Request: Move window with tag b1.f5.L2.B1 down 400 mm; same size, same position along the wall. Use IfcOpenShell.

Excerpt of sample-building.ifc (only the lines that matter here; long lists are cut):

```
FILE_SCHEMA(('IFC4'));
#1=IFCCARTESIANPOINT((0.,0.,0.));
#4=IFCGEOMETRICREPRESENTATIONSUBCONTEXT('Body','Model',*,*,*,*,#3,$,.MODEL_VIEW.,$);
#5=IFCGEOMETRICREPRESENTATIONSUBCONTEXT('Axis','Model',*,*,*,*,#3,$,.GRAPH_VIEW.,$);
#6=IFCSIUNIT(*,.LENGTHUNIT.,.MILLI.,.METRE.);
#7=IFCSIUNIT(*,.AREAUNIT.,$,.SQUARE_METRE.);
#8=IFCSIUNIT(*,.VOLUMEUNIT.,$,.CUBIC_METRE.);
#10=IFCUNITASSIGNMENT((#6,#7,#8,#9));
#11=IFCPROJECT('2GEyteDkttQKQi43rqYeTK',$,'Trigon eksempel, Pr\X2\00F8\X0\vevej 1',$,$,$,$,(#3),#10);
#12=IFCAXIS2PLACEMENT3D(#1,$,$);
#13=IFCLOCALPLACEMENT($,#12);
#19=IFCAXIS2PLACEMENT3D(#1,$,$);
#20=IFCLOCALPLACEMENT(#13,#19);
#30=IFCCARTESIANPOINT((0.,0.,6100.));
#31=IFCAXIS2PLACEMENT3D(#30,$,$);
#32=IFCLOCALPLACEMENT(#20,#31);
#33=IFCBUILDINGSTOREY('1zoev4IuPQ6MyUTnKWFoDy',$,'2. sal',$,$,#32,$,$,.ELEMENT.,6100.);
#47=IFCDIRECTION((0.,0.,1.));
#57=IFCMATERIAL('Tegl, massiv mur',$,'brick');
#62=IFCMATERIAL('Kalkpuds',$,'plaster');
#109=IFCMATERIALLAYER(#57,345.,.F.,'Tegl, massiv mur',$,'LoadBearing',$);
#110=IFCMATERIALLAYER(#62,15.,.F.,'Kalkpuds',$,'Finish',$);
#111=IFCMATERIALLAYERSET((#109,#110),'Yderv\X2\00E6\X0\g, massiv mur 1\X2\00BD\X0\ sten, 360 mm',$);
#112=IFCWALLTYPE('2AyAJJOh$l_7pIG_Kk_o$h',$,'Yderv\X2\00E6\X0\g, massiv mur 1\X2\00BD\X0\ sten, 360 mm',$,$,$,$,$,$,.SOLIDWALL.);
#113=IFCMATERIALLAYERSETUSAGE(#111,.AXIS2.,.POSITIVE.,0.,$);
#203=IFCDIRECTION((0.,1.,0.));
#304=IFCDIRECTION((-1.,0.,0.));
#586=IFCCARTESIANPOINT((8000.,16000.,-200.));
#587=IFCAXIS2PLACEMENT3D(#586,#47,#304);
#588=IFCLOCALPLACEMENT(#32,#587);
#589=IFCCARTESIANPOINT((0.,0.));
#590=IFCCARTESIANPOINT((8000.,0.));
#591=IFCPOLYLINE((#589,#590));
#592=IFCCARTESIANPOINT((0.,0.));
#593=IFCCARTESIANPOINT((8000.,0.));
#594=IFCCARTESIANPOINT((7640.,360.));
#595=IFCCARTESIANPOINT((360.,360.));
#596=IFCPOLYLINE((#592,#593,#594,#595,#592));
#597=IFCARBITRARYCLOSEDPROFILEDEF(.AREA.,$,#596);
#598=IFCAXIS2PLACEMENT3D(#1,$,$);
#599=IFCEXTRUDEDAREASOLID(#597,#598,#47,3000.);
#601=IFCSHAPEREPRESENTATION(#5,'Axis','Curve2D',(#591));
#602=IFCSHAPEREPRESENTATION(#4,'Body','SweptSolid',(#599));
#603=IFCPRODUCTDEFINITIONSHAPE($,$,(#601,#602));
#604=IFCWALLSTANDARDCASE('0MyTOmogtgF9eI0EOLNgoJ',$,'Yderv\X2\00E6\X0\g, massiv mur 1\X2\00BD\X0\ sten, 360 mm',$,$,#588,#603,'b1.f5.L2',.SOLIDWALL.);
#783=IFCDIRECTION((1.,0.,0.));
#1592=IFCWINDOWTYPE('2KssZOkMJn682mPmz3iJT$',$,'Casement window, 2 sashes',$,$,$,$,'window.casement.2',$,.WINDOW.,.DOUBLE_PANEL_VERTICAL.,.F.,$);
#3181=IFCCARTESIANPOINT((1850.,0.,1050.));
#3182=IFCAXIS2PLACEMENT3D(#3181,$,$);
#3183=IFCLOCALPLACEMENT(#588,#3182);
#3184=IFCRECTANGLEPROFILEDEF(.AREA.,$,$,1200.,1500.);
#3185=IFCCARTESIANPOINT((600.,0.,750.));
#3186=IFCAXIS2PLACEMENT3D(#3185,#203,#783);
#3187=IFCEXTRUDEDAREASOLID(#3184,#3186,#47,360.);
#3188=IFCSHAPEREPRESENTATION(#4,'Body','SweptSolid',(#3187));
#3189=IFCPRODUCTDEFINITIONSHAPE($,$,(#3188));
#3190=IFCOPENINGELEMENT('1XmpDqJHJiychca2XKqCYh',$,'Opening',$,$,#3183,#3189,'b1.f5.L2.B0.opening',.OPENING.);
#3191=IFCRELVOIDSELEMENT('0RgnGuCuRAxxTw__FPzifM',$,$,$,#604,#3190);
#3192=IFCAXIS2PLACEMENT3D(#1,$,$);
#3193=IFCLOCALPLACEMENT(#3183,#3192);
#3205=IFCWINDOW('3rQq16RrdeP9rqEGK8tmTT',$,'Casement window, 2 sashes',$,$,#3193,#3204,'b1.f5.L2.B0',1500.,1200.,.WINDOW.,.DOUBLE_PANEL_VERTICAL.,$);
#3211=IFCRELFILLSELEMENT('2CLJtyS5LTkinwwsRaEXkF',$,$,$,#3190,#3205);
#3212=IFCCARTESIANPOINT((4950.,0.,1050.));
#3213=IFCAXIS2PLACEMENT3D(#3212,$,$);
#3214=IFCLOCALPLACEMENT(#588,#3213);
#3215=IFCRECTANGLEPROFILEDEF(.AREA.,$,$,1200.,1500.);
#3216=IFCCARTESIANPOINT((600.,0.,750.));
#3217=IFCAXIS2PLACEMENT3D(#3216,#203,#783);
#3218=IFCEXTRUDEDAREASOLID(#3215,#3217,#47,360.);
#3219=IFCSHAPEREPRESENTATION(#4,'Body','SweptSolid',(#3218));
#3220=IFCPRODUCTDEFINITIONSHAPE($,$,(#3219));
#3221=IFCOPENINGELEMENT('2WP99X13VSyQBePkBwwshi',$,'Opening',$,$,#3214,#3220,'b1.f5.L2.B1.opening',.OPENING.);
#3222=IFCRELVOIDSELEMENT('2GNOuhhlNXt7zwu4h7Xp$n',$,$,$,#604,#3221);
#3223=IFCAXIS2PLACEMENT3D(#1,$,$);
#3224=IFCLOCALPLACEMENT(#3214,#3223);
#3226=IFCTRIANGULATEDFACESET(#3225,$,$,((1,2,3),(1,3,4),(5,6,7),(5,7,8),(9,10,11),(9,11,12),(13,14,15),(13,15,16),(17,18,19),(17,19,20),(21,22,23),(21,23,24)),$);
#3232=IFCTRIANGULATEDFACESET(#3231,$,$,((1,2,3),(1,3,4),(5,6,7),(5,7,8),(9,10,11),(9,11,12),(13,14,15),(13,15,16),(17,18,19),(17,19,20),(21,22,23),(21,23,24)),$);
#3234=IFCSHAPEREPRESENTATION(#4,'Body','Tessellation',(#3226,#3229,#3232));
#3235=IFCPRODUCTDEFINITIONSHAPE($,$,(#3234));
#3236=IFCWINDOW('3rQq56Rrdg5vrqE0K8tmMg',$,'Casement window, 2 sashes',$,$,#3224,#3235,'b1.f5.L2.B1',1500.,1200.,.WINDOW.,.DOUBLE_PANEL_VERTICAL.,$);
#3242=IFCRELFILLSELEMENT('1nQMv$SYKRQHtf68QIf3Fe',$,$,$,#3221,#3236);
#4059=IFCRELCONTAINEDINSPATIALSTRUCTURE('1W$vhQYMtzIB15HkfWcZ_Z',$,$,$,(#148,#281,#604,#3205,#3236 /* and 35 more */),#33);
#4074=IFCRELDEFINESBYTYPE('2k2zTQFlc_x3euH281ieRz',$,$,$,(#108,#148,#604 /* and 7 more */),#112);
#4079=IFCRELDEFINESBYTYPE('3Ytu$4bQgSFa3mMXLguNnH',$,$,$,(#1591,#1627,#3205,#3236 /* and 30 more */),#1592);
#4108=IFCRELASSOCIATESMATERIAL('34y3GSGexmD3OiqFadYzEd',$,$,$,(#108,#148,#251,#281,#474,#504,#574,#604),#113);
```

```python
import numpy as np
import ifcopenshell
import ifcopenshell.api.geometry
import ifcopenshell.util.placement
import ifcopenshell.util.unit

model = ifcopenshell.open("sample-building.ifc")
unit_scale = ifcopenshell.util.unit.calculate_unit_scale(model)

window = model.by_guid("3rQq56Rrdg5vrqE0K8tmMg")
opening = window.FillsVoids[0].RelatingOpeningElement
dz = -0.4 / unit_scale

shift = np.array([0.0, 0.0, dz])
# The window is placed relative to its opening, so it follows when the opening moves.
matrix = ifcopenshell.util.placement.get_local_placement(opening.ObjectPlacement)
matrix[:3, 3] += shift
ifcopenshell.api.geometry.edit_object_placement(
    model, product=opening, matrix=matrix, is_si=False, should_transform_children=True
)

print(f"moved by {dz * unit_scale:+.3f} m")

model.write("sample-building_edited.ifc")
```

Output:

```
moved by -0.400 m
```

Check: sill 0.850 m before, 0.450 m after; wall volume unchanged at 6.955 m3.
